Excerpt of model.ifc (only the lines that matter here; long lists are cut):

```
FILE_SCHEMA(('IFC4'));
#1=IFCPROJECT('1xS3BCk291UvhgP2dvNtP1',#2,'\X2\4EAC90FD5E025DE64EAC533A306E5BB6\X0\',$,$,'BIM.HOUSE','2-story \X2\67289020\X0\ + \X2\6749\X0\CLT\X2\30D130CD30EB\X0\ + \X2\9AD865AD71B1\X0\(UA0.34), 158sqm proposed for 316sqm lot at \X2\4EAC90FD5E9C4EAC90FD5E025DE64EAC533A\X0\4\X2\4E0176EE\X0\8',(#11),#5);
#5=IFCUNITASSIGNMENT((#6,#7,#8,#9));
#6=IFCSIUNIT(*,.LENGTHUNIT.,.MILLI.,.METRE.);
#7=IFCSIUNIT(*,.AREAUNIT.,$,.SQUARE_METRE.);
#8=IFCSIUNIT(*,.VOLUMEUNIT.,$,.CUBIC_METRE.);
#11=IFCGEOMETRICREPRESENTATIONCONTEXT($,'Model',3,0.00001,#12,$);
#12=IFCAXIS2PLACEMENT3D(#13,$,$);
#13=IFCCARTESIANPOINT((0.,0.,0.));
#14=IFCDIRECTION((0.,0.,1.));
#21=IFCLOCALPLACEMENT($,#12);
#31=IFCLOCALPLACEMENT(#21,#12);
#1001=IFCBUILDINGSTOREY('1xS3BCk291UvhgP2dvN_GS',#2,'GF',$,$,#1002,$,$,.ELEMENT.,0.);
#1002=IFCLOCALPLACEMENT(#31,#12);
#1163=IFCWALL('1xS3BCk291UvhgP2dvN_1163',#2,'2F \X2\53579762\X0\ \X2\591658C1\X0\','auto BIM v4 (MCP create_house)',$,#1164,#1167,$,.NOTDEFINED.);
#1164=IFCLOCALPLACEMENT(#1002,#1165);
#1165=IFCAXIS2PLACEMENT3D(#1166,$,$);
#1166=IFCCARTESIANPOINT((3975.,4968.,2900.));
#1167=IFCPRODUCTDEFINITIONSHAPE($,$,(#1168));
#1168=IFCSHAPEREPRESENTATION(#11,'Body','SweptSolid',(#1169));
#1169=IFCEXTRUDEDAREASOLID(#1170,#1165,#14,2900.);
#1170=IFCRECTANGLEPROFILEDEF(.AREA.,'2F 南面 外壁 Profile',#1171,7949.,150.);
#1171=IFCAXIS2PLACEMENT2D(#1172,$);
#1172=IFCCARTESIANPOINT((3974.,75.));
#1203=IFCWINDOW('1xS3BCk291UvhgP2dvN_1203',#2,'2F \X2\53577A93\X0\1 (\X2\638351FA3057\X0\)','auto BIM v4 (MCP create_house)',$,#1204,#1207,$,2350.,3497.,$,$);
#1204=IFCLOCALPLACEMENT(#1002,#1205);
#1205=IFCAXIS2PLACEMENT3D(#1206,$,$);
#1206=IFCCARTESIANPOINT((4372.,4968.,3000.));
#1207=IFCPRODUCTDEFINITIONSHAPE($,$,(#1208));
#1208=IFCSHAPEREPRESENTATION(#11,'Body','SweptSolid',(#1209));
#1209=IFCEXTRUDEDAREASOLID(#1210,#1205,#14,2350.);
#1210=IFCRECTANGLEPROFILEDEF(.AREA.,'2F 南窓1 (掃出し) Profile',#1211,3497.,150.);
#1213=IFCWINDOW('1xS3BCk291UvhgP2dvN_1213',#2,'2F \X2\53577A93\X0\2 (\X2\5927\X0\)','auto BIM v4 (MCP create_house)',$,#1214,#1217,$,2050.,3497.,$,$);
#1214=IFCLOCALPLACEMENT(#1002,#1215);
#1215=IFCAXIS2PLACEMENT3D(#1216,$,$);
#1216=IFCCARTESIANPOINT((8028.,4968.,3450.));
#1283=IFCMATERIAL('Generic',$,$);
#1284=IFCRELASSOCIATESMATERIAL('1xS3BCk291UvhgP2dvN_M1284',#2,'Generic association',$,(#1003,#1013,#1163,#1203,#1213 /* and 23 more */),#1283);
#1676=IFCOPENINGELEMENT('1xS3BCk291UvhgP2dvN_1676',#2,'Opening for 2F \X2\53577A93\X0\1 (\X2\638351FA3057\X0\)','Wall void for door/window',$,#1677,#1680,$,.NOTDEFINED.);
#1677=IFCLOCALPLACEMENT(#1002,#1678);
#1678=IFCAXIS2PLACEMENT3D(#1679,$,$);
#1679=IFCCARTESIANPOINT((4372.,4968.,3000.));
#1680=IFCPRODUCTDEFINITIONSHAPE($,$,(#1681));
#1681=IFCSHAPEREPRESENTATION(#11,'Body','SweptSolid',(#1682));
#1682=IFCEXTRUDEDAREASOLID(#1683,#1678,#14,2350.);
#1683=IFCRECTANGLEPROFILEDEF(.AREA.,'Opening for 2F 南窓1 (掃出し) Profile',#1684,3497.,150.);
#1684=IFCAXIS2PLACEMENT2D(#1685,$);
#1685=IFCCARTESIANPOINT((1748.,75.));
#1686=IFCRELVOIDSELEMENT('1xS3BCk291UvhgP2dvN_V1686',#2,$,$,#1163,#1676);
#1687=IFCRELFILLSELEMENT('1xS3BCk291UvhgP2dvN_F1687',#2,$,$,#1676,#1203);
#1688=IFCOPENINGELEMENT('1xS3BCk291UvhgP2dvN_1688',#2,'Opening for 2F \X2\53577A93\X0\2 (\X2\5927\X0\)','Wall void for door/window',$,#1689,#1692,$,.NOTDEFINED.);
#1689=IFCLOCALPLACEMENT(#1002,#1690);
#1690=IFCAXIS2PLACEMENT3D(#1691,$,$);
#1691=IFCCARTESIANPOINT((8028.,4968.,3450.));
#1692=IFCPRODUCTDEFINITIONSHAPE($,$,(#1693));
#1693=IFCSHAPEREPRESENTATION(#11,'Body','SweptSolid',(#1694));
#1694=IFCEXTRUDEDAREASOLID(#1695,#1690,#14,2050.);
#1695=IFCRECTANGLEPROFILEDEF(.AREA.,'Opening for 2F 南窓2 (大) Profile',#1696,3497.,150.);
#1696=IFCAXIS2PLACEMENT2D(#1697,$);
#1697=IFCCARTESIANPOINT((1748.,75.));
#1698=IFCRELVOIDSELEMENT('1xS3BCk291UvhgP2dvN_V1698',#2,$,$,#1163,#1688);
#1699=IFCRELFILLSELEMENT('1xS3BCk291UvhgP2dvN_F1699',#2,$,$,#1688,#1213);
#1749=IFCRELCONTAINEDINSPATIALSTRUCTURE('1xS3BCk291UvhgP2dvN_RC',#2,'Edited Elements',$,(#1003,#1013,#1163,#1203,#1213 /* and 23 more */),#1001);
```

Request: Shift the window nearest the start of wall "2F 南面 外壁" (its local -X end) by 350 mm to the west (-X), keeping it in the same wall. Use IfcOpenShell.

```python
import ifcopenshell
import ifcopenshell.api.geometry
import ifcopenshell.util.placement
import ifcopenshell.util.unit

model = ifcopenshell.open("model.ifc")
unit_scale = ifcopenshell.util.unit.calculate_unit_scale(model)

window = model.by_id(1203)
opening = window.FillsVoids[0].RelatingOpeningElement
wall = opening.VoidsElements[0].RelatingBuildingElement

wall_matrix = ifcopenshell.util.placement.get_local_placement(wall.ObjectPlacement)
shift = wall_matrix[:3, 0] * -0.35 / unit_scale
before = ifcopenshell.util.placement.get_local_placement(window.ObjectPlacement)[:3, 3].copy()

# The window is not placed relative to its opening, so move both.
for product in (opening, window):
    matrix = ifcopenshell.util.placement.get_local_placement(product.ObjectPlacement)
    matrix[:3, 3] += shift
    ifcopenshell.api.geometry.edit_object_placement(model, product=product, matrix=matrix, is_si=False)

after = ifcopenshell.util.placement.get_local_placement(window.ObjectPlacement)[:3, 3]
print("window moved by", (after - before).round(3) + 0.0)

model.write("model_v2.ifc")
```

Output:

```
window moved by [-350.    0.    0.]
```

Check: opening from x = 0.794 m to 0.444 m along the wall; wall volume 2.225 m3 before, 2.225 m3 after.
